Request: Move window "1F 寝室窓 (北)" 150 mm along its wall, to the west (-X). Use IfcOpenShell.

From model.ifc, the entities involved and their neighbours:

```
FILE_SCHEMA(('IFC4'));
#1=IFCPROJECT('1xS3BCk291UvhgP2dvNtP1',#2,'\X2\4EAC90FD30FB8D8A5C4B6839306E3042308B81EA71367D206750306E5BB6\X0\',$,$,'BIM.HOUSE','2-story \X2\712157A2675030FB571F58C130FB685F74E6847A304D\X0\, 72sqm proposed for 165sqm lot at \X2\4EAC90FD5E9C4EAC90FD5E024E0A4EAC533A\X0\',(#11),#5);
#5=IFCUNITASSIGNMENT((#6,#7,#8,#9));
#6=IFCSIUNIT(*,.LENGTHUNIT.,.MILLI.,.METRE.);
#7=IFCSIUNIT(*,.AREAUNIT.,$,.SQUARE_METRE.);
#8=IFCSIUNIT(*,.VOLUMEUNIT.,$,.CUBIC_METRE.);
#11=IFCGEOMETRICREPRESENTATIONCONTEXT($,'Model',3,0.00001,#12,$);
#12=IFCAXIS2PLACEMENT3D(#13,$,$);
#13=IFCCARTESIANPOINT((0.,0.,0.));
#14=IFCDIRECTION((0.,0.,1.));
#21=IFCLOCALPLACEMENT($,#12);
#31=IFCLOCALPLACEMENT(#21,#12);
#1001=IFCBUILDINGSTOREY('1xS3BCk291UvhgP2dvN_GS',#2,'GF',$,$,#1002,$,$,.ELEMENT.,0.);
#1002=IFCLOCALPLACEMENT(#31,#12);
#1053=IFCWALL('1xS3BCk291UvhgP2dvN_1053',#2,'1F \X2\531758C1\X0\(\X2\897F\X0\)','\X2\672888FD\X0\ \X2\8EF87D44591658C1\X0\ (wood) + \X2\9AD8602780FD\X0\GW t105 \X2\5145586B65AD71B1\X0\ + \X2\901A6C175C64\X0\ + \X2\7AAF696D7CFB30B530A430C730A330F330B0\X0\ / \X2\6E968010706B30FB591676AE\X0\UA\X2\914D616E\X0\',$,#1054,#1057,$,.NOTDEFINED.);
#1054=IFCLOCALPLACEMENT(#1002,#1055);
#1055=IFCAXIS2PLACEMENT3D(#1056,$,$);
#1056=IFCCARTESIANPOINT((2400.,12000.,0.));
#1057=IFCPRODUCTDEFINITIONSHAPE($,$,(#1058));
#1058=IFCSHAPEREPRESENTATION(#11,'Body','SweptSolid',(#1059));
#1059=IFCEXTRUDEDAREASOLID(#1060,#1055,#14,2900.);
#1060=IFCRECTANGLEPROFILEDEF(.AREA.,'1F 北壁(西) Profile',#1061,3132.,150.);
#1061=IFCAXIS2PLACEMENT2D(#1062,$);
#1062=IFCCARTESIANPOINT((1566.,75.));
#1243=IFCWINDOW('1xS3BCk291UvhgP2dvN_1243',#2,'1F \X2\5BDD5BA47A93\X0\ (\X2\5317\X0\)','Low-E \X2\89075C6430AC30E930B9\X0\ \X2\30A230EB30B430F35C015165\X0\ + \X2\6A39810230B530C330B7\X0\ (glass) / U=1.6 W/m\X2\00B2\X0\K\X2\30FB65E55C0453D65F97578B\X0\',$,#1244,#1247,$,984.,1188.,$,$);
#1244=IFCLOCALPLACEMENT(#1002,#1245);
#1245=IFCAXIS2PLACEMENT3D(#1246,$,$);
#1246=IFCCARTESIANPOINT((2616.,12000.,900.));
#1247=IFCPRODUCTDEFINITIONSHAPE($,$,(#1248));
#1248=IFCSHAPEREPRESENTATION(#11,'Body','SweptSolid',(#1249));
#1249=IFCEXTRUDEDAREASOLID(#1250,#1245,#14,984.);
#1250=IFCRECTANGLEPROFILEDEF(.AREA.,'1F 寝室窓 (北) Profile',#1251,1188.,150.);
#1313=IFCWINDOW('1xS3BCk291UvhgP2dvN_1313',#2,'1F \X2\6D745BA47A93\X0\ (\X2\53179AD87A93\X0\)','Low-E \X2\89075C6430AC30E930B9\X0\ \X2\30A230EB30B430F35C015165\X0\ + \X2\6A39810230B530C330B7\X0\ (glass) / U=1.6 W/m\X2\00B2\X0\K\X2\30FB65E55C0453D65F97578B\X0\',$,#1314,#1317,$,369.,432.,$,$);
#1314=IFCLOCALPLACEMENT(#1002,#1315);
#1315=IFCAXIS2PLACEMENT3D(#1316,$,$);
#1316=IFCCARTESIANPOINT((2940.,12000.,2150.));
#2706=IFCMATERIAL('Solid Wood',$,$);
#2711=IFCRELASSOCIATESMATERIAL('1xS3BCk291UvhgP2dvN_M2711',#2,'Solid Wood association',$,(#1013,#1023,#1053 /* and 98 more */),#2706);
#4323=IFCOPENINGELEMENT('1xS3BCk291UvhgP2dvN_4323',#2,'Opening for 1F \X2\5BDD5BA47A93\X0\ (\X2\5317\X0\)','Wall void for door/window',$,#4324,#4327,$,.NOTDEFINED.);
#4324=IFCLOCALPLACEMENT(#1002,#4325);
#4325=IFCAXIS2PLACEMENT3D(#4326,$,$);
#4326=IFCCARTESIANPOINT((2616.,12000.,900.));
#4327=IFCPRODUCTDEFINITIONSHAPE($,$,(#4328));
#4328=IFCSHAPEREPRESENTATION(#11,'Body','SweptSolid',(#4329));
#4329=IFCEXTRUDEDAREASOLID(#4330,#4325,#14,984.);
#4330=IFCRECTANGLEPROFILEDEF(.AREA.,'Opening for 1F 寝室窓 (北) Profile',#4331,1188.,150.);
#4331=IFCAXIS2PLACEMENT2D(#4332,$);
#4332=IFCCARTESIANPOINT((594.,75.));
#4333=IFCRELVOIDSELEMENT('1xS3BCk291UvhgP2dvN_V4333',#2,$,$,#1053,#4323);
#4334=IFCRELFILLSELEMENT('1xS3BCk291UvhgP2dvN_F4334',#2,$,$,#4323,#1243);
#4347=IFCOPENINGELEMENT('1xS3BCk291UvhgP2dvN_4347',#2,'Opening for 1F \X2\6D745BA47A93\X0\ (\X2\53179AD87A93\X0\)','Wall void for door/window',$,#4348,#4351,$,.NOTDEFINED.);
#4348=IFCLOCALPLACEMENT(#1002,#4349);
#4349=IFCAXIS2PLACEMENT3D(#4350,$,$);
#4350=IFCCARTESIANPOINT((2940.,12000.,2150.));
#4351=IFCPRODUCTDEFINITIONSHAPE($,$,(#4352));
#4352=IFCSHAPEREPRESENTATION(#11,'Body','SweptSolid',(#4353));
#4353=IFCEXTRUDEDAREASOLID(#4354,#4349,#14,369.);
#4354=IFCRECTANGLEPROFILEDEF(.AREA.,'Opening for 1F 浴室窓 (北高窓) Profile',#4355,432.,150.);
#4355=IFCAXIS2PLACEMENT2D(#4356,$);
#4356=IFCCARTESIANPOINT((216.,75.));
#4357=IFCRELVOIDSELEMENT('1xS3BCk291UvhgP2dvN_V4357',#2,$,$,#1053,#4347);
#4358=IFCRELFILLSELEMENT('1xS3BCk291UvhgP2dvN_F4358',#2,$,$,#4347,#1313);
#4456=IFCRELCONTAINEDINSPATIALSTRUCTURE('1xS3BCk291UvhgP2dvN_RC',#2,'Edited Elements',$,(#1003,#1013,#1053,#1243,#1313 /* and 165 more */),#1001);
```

```python
import ifcopenshell
import ifcopenshell.api.geometry
import ifcopenshell.util.placement
import ifcopenshell.util.unit

model = ifcopenshell.open("model.ifc")
unit_scale = ifcopenshell.util.unit.calculate_unit_scale(model)

window = model.by_guid("1xS3BCk291UvhgP2dvN_1243")
opening = window.FillsVoids[0].RelatingOpeningElement
wall = opening.VoidsElements[0].RelatingBuildingElement

wall_matrix = ifcopenshell.util.placement.get_local_placement(wall.ObjectPlacement)
shift = wall_matrix[:3, 0] * -0.15 / unit_scale
before = ifcopenshell.util.placement.get_local_placement(window.ObjectPlacement)[:3, 3].copy()

# The window is not placed relative to its opening, so move both.
for product in (opening, window):
    matrix = ifcopenshell.util.placement.get_local_placement(product.ObjectPlacement)
    matrix[:3, 3] += shift
    ifcopenshell.api.geometry.edit_object_placement(model, product=product, matrix=matrix, is_si=False)

after = ifcopenshell.util.placement.get_local_placement(window.ObjectPlacement)[:3, 3]
print("window moved by", (after - before).round(3) + 0.0)

model.write("model_updated.ifc")
```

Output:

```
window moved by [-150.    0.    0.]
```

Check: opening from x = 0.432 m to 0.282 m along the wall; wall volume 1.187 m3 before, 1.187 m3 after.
